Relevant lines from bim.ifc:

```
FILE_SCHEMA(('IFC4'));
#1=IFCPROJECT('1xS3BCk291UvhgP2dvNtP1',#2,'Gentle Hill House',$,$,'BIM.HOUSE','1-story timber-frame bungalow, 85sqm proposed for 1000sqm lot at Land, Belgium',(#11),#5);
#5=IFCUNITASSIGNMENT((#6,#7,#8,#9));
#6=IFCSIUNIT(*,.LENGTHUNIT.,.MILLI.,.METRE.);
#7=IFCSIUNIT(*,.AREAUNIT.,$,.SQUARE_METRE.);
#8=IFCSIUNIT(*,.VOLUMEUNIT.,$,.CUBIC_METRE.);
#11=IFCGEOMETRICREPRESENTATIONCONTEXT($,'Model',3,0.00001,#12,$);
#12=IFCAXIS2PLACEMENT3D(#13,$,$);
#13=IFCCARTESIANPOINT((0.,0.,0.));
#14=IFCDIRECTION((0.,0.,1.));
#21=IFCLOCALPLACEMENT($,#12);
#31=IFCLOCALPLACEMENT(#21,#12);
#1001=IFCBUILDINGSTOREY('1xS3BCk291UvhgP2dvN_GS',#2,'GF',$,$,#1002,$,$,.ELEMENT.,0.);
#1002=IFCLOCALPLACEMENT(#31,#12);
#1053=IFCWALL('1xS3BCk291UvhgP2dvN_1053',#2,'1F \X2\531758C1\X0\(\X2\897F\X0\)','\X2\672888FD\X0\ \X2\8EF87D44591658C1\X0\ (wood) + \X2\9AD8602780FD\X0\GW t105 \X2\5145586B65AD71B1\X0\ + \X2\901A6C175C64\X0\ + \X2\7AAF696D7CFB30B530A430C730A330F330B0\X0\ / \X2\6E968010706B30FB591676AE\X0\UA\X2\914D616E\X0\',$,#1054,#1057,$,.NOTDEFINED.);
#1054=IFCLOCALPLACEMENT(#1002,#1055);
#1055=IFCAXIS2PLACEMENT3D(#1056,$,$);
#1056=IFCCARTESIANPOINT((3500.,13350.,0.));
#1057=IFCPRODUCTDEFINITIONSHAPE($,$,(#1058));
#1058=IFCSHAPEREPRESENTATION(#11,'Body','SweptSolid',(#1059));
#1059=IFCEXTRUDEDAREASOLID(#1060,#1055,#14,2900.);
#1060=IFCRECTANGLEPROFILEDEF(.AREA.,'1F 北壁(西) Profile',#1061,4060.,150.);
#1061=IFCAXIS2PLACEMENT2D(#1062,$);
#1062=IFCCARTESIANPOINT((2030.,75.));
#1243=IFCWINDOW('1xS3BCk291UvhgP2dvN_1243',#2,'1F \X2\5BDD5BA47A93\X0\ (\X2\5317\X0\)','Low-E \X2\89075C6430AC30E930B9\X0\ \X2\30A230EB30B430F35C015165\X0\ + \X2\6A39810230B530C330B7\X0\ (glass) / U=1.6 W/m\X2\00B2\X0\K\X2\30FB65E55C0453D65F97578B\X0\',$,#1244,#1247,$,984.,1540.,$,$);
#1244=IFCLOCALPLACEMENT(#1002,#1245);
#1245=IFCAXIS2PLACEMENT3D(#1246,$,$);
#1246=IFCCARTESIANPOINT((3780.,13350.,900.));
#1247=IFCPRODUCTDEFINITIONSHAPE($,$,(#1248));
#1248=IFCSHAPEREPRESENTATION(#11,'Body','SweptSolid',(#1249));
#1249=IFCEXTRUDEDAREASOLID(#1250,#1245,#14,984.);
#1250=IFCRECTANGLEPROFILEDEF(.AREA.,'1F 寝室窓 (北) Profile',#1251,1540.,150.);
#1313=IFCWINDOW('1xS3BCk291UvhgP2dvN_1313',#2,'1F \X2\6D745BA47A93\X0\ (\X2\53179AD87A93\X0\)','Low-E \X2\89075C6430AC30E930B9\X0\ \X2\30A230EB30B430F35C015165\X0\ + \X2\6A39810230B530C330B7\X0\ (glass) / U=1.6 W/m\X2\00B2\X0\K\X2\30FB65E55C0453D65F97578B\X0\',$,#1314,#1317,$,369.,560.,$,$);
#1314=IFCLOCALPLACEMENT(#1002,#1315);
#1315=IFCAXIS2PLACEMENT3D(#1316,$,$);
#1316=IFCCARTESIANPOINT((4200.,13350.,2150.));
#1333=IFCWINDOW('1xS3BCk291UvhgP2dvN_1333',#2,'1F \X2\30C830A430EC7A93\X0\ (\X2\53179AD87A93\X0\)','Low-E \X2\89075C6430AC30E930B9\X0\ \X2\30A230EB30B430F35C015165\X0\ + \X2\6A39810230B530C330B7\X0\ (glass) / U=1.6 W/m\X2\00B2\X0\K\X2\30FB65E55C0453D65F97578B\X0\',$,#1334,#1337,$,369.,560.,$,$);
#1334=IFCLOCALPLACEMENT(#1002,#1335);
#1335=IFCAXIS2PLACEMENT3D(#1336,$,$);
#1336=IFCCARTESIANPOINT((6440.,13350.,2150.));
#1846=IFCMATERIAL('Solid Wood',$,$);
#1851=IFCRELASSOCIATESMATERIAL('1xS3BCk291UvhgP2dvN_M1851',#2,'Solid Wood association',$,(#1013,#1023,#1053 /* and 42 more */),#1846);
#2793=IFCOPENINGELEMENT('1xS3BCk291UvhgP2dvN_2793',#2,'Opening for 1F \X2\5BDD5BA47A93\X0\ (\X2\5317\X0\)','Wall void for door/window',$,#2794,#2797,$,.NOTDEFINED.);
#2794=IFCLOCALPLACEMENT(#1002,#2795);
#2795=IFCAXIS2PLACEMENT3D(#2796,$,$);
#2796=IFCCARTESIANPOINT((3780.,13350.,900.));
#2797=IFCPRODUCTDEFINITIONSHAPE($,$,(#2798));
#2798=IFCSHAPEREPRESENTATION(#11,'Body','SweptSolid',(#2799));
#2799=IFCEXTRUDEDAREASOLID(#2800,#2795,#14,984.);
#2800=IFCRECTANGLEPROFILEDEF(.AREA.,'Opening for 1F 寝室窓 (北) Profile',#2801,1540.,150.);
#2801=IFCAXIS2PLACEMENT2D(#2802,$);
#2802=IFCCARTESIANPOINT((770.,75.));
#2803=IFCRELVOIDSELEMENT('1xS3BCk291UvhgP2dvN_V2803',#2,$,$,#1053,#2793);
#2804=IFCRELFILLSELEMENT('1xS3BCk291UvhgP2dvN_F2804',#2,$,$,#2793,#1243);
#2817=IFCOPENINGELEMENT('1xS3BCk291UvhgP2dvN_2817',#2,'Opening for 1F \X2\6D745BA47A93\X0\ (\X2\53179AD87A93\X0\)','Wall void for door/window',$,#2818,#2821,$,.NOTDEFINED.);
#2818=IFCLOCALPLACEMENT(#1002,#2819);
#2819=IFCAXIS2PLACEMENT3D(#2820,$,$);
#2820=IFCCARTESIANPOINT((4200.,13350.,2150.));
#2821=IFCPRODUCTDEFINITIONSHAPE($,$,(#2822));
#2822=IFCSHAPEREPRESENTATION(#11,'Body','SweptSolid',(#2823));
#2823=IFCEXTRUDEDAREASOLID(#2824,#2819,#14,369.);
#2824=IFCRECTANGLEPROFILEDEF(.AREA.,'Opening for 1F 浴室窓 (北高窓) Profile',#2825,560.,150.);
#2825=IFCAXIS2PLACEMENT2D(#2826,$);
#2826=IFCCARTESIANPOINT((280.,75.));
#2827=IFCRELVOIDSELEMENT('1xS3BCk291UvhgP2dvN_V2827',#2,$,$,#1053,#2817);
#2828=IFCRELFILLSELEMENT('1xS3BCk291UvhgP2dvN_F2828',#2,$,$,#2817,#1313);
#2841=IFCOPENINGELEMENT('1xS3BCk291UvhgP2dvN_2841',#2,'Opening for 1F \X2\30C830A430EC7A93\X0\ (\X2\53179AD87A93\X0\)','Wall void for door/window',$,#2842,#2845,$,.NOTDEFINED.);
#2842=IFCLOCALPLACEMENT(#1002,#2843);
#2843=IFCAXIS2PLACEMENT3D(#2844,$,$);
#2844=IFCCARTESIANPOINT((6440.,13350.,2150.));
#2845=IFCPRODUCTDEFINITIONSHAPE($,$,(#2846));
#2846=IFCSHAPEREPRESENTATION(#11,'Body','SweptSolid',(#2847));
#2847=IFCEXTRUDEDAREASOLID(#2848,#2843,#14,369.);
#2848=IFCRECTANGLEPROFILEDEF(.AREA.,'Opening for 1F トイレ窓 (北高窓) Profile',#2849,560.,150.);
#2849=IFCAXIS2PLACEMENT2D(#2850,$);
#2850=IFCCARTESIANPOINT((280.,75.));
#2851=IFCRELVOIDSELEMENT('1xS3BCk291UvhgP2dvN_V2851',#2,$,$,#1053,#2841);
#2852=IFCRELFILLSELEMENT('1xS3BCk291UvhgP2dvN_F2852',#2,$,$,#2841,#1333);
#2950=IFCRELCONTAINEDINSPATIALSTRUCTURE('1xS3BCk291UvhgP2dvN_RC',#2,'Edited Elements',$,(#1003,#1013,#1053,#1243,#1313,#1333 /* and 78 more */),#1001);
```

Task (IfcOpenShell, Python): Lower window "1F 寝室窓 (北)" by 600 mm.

```python
import numpy as np
import ifcopenshell
import ifcopenshell.api.geometry
import ifcopenshell.util.placement
import ifcopenshell.util.unit

model = ifcopenshell.open("bim.ifc")
unit_scale = ifcopenshell.util.unit.calculate_unit_scale(model)

window = model.by_guid("1xS3BCk291UvhgP2dvN_1243")
opening = window.FillsVoids[0].RelatingOpeningElement
dz = -600.0

shift = np.array([0.0, 0.0, dz])
# The window is not placed relative to its opening, so move both.
for product in (opening, window):
    matrix = ifcopenshell.util.placement.get_local_placement(product.ObjectPlacement)
    matrix[:3, 3] += shift
    ifcopenshell.api.geometry.edit_object_placement(model, product=product, matrix=matrix, is_si=False)

print(f"moved by {dz * unit_scale:+.3f} m")

model.write("bim-out.ifc")
```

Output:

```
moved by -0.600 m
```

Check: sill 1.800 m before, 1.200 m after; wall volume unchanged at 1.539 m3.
